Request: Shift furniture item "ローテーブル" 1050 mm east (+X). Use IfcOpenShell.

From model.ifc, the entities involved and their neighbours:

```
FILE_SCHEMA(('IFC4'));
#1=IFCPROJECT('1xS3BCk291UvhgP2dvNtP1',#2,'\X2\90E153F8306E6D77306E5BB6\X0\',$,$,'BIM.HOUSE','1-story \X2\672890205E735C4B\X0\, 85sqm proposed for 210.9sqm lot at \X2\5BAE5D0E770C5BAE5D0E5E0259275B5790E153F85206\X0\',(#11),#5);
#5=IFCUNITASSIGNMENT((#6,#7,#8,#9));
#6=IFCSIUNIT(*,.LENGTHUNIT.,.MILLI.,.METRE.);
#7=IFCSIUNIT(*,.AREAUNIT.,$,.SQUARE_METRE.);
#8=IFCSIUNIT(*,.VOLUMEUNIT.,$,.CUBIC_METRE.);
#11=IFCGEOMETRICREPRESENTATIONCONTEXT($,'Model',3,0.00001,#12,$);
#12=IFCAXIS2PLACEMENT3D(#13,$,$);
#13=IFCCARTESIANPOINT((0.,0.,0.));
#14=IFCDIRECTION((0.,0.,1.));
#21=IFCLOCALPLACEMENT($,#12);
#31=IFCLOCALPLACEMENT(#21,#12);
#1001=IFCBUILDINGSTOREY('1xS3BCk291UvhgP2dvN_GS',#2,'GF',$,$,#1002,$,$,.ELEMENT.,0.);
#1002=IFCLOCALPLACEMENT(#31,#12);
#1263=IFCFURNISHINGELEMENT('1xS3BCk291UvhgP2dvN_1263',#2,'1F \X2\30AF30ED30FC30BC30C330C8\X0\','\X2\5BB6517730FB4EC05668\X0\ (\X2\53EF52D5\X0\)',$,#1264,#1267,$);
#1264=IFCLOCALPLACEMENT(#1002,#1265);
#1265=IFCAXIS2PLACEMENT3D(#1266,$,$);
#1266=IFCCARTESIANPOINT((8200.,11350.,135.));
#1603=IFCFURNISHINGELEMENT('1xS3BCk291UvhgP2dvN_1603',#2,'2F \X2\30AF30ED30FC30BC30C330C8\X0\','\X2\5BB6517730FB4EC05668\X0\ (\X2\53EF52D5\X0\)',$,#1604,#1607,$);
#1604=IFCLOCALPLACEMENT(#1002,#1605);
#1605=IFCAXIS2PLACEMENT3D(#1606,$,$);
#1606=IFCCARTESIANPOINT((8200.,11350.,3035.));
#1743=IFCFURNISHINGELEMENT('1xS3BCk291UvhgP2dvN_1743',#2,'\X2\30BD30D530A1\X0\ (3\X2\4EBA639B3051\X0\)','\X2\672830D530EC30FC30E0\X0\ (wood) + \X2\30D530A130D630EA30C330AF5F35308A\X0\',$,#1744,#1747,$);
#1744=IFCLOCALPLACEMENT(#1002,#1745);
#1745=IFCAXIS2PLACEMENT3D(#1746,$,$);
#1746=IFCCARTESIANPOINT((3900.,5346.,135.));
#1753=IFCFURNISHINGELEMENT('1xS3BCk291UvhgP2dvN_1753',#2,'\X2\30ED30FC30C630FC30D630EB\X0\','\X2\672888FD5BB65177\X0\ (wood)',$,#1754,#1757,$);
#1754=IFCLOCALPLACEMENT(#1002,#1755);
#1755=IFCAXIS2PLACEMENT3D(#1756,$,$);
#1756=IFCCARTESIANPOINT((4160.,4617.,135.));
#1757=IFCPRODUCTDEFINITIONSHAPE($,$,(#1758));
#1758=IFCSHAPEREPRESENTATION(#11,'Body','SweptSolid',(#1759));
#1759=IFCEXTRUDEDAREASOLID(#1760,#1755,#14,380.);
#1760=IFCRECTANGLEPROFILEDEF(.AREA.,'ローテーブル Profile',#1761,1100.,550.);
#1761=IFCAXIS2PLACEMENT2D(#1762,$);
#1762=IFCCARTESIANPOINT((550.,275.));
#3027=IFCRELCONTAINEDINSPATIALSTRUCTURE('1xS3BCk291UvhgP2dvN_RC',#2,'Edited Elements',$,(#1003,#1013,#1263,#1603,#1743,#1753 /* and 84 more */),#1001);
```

```python
import ifcopenshell
import ifcopenshell.api.geometry
import ifcopenshell.util.placement
import ifcopenshell.util.unit

model = ifcopenshell.open("model.ifc")
unit_scale = ifcopenshell.util.unit.calculate_unit_scale(model)

item = model.by_guid("1xS3BCk291UvhgP2dvN_1753")
matrix = ifcopenshell.util.placement.get_local_placement(item.ObjectPlacement)
matrix[0, 3] += 1.05 / unit_scale
ifcopenshell.api.geometry.edit_object_placement(model, product=item, matrix=matrix, is_si=False)

print(ifcopenshell.util.placement.get_local_placement(item.ObjectPlacement).round(3) + 0.0)

model.write("model-out.ifc")
```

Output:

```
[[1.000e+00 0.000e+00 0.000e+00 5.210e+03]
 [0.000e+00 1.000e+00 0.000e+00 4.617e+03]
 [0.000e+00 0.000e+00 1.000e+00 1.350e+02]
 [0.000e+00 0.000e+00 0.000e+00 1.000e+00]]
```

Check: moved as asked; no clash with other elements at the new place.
